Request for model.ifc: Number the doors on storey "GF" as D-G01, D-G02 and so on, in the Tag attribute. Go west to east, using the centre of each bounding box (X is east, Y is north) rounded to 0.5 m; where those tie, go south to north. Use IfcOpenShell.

First a look at what the model holds.

```python
import ifcopenshell
import ifcopenshell.util.element
import ifcopenshell.util.placement

model = ifcopenshell.open("model.ifc")
print(model.schema)
storey = next(s for s in model.by_type("IfcBuildingStorey") if s.Name == "GF")
doors = [e for e in ifcopenshell.util.element.get_decomposition(storey) if e.is_a("IfcDoor")]
for e in sorted(doors, key=lambda e: e.id()):
    origin = ifcopenshell.util.placement.get_local_placement(e.ObjectPlacement)[:3, 3]
    print(e.id(), e.Tag, e.Name, origin.round(2) + 0.0, sep=" | ")
```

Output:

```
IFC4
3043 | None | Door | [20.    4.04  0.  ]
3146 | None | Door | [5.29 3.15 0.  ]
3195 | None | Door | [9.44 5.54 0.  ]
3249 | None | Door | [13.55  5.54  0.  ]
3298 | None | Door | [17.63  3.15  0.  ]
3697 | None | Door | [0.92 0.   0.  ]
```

```python
import ifcopenshell
import ifcopenshell.geom
import ifcopenshell.util.element
import ifcopenshell.util.shape

model = ifcopenshell.open("model.ifc")
settings = ifcopenshell.geom.settings()
settings.set("use-world-coords", True)


def centre(element):
    shape = ifcopenshell.geom.create_shape(settings, element)
    return ifcopenshell.util.shape.get_bbox_centroid(shape.geometry)


storey = next(s for s in model.by_type("IfcBuildingStorey") if s.Name == "GF")
doors = [e for e in ifcopenshell.util.element.get_decomposition(storey) if e.is_a("IfcDoor")]

# Insertion points can sit at a corner or the storey origin, so sort by the geometry (in metres).
centres = {e: centre(e) for e in doors}
doors.sort(key=lambda e: (round(centres[e][0] / 0.5), centres[e][1]))

for i, e in enumerate(doors, start=1):
    number = f"D-G{i:02d}"
    e.Tag = number
    print(e.id(), number)

model.write("model_v2.ifc")
```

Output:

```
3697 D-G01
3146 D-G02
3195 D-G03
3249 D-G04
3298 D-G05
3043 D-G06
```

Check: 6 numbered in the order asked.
